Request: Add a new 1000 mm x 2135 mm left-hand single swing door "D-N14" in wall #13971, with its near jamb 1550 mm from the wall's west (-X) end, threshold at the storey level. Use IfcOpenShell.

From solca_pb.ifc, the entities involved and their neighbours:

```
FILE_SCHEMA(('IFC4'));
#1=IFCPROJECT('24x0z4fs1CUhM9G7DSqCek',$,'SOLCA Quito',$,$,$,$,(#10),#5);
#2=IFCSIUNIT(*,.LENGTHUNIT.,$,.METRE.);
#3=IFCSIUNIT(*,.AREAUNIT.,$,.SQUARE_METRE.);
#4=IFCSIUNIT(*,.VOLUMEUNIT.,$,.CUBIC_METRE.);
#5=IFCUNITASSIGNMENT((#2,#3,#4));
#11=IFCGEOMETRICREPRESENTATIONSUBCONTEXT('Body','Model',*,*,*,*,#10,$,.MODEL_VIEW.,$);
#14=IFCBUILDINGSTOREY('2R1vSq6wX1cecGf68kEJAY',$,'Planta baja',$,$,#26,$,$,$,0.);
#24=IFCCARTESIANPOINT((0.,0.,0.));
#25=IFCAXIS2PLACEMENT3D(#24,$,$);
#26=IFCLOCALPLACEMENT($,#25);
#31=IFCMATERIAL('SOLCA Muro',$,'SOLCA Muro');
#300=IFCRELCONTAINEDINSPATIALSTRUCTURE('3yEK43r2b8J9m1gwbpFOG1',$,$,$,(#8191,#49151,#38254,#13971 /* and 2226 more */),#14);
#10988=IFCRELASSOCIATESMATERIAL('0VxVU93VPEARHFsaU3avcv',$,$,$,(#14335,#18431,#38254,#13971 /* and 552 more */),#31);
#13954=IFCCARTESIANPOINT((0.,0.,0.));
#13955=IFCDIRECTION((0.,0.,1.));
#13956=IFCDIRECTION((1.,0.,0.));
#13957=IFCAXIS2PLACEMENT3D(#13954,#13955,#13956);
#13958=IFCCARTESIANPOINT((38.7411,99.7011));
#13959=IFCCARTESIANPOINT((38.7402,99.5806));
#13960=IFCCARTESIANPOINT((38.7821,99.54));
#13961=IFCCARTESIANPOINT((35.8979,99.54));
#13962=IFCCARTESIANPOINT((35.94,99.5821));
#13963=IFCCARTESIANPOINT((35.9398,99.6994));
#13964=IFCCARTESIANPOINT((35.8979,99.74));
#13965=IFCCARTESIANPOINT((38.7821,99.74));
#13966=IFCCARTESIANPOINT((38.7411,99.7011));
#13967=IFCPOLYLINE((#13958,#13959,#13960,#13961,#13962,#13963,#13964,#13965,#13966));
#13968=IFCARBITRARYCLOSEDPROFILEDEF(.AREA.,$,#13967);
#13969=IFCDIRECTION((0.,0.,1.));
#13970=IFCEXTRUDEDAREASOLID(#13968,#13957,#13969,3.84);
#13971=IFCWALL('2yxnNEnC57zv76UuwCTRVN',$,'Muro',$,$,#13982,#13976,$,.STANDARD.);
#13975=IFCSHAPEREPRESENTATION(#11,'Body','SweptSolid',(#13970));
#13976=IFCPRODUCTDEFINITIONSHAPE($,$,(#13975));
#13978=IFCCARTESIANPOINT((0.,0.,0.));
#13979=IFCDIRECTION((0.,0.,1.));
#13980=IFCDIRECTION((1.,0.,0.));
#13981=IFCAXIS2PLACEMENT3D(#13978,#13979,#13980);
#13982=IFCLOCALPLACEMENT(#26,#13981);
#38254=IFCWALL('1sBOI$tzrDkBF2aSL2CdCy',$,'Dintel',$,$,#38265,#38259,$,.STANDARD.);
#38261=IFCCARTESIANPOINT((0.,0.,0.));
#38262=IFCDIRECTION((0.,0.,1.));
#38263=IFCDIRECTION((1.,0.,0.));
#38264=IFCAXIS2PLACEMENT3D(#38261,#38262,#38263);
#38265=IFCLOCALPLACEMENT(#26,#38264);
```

```python
import numpy as np
import ifcopenshell
import ifcopenshell.api.feature
import ifcopenshell.api.geometry
import ifcopenshell.api.root
import ifcopenshell.api.spatial
import ifcopenshell.geom
import ifcopenshell.util.element
import ifcopenshell.util.placement
import ifcopenshell.util.representation
import ifcopenshell.util.shape
import ifcopenshell.util.unit

model = ifcopenshell.open("solca_pb.ifc")
unit_scale = ifcopenshell.util.unit.calculate_unit_scale(model)
settings = ifcopenshell.geom.settings()


def volume(element):
    """Net volume in cubic metres, openings subtracted."""
    shape = ifcopenshell.geom.create_shape(settings, element)
    return ifcopenshell.util.shape.get_volume(shape.geometry)


wall = model.by_guid("2yxnNEnC57zv76UuwCTRVN")
storey = ifcopenshell.util.element.get_container(wall, ifc_class="IfcBuildingStorey")
context = ifcopenshell.util.representation.get_context(model, "Model", "Body", "MODEL_VIEW")
before = volume(wall)

width, height, from_end, sill = 1, 2.135, 1.55, 0.0  # metres

# The wall runs along its own X axis, and the end named is its -X end.
wall_shape = ifcopenshell.geom.create_shape(settings, wall)
x, y, z = ifcopenshell.util.shape.get_vertices(wall_shape.geometry).T
start = x.min() + from_end
face, thickness = float(y.min()), float(y.max() - y.min())
wall_matrix = ifcopenshell.util.placement.get_local_placement(wall.ObjectPlacement)
level = ifcopenshell.util.placement.get_local_placement(storey.ObjectPlacement)[2, 3]


def in_wall(x, y):
    """Placement at x, y metres in the wall's axes, at sill height."""
    matrix = wall_matrix.copy()
    matrix[:, 3] = wall_matrix @ np.array([x / unit_scale, y / unit_scale, 0.0, 1.0])
    matrix[2, 3] = level + sill / unit_scale
    return matrix


# Opening: a box that overshoots both wall faces by 50 mm.
opening = ifcopenshell.api.root.create_entity(model, ifc_class="IfcOpeningElement", predefined_type="OPENING")
box = ifcopenshell.api.geometry.add_wall_representation(
    model, context=context, length=width, height=height, thickness=thickness + 0.1
)
ifcopenshell.api.geometry.assign_representation(model, product=opening, representation=box)
ifcopenshell.api.geometry.edit_object_placement(model, product=opening, matrix=in_wall(start, face - 0.05), is_si=False)
ifcopenshell.api.feature.add_feature(model, feature=opening, element=wall)

door = ifcopenshell.api.root.create_entity(model, ifc_class="IfcDoor", name="D-N14", predefined_type="DOOR")
door.OverallWidth, door.OverallHeight = width / unit_scale, height / unit_scale
door.OperationType = "SINGLE_SWING_LEFT"
body = ifcopenshell.api.geometry.add_door_representation(
    model,
    context=context,
    overall_width=door.OverallWidth,
    overall_height=door.OverallHeight,
    operation_type="SINGLE_SWING_LEFT",
    lining_properties={"LiningDepth": thickness / unit_scale, "ThresholdDepth": thickness / unit_scale},
)
ifcopenshell.api.geometry.assign_representation(model, product=door, representation=body)
ifcopenshell.api.spatial.assign_container(model, products=[door], relating_structure=storey)
ifcopenshell.api.feature.add_filling(model, opening=opening, element=door)

# The lining spans the wall, so the door starts at the wall face.
ifcopenshell.api.geometry.edit_object_placement(model, product=door, matrix=in_wall(start, face), is_si=False)

after = volume(wall)

print(f"wall volume {before:.3f} -> {after:.3f} m3")

model.write("solca_pb_rev.ifc")
```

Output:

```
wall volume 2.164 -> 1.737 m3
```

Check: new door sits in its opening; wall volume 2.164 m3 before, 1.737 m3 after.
